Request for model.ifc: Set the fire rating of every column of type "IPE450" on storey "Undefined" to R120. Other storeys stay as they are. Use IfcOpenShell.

First a look at what the model holds.

```python
import ifcopenshell
import ifcopenshell.util.element

model = ifcopenshell.open("model.ifc")
print(model.schema)
storey = next(s for s in model.by_type("IfcBuildingStorey") if s.Name == "Undefined")
columns = [e for e in ifcopenshell.util.element.get_decomposition(storey) if e.is_a("IfcColumn")]
seen = {}
for e in columns:
    element_type = ifcopenshell.util.element.get_type(e)
    key = (element_type.Name if element_type != e and element_type else None, ifcopenshell.util.element.get_pset(e, "Pset_ColumnCommon", "FireRating"))
    seen[key] = seen.get(key, 0) + 1
for (name, value), count in sorted(seen.items(), key=str):
    print(count, "x", name, "|", value)
```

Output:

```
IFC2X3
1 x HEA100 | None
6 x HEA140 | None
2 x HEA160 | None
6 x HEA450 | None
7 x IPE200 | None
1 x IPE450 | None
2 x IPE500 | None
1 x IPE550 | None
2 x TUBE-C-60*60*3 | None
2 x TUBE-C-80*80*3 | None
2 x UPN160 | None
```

```python
import ifcopenshell
import ifcopenshell.api.pset
import ifcopenshell.util.element

model = ifcopenshell.open("model.ifc")

storey = next(s for s in model.by_type("IfcBuildingStorey") if s.Name == "Undefined")
columns = [e for e in ifcopenshell.util.element.get_decomposition(storey) if e.is_a("IfcColumn")]

count = 0
for e in columns:
    element_type = ifcopenshell.util.element.get_type(e)
    if element_type in (None, e) or element_type.Name != "IPE450":
        continue
    # add_pset returns the element's existing set when there is one.
    pset = ifcopenshell.api.pset.add_pset(model, product=e, name="Pset_ColumnCommon")
    ifcopenshell.api.pset.edit_pset(model, pset=pset, properties={"FireRating": "R120"})
    count += 1

print(count, "columns updated")

model.write("model_updated.ifc")
```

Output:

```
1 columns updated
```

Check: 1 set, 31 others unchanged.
